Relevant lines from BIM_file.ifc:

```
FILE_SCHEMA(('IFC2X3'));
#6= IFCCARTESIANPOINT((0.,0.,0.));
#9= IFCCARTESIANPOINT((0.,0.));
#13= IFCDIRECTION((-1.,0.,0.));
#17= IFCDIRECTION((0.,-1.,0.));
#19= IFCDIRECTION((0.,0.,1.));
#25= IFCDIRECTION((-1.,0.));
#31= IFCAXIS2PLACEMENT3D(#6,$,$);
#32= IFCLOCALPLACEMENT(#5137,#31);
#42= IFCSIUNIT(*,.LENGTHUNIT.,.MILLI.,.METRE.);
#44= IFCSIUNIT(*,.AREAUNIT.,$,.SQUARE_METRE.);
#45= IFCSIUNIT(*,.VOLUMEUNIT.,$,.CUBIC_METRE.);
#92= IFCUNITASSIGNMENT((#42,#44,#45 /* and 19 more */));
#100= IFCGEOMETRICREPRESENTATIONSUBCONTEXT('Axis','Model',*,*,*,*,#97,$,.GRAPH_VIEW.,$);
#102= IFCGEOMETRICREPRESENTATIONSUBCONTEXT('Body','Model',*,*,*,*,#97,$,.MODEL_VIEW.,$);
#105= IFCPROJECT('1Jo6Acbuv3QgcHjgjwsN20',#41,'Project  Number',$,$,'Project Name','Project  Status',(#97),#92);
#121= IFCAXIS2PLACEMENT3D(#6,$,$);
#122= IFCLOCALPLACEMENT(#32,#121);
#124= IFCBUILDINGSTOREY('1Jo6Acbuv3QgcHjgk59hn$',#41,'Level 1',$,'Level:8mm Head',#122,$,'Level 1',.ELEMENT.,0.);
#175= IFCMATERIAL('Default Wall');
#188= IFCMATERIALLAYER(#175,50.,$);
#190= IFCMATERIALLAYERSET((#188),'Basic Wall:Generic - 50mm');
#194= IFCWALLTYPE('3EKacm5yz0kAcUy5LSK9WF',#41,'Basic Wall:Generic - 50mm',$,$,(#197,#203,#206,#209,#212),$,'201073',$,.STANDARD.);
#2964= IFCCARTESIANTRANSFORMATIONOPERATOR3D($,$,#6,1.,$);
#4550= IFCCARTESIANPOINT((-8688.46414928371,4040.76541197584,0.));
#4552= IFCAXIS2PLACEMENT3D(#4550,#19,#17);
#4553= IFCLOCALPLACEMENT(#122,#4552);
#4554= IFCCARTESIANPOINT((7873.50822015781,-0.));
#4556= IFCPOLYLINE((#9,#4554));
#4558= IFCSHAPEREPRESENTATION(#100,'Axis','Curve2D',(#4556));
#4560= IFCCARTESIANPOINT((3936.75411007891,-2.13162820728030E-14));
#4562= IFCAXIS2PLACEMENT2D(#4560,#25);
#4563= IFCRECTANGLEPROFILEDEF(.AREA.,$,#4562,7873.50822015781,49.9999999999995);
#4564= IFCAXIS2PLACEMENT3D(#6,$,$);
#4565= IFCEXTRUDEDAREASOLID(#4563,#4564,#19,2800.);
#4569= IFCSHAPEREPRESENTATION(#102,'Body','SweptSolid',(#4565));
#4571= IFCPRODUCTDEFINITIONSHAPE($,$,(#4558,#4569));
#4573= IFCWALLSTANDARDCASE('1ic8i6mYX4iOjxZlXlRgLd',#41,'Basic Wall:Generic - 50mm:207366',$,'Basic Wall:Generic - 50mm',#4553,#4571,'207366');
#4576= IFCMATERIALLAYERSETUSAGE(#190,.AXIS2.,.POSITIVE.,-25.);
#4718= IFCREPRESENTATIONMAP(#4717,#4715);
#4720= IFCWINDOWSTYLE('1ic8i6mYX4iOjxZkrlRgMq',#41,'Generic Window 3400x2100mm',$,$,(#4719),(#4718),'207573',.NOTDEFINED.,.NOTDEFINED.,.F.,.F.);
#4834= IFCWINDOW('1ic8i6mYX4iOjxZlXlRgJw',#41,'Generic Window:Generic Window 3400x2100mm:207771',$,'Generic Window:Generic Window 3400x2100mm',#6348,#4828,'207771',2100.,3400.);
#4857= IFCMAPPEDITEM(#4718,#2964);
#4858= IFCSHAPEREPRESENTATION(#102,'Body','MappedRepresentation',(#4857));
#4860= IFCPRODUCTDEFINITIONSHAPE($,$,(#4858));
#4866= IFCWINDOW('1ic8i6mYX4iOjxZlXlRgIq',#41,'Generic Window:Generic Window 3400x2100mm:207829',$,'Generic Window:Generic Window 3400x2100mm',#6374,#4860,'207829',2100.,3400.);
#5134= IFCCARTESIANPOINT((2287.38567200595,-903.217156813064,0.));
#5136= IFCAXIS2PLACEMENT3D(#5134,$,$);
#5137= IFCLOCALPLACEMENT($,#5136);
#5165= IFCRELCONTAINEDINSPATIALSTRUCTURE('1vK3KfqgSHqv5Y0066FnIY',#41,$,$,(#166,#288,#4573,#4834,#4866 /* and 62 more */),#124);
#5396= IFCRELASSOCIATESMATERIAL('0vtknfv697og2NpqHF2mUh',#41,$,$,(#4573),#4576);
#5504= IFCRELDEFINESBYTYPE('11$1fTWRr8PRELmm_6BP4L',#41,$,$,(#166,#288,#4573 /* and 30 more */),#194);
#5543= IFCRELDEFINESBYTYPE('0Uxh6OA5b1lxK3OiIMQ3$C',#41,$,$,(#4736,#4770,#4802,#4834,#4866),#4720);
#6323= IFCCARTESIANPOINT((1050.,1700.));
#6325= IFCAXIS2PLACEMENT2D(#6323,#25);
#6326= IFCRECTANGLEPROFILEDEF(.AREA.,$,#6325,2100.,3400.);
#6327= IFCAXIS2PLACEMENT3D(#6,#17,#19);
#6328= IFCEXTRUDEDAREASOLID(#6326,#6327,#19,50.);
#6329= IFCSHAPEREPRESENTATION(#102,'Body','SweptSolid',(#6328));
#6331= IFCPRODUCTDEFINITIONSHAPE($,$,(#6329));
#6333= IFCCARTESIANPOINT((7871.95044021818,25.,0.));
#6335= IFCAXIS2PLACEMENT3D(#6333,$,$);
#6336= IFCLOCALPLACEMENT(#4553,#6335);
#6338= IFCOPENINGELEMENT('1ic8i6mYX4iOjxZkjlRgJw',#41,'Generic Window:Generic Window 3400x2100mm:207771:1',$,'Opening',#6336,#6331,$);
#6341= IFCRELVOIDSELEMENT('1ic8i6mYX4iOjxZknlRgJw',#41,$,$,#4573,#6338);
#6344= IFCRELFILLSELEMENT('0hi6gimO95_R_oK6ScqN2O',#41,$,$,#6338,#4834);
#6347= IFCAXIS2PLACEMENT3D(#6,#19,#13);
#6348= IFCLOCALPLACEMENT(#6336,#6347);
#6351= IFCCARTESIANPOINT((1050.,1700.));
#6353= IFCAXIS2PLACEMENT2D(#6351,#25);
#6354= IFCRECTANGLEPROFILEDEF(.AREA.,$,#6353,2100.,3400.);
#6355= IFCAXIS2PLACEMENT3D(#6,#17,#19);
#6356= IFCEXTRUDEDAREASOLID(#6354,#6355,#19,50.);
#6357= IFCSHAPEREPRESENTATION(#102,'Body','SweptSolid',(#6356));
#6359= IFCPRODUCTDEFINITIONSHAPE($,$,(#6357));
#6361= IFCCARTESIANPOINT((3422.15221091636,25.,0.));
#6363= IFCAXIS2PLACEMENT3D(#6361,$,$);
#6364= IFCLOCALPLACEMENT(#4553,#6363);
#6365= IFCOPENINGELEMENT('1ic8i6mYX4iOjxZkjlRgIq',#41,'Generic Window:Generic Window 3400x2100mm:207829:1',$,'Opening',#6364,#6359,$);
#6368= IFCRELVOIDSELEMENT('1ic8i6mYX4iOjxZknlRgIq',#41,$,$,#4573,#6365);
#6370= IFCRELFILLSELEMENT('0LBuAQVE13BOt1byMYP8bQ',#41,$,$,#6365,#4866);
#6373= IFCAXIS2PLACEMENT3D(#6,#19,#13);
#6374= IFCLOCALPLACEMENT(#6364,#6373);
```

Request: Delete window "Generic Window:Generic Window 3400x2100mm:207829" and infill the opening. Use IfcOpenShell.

```python
import ifcopenshell
import ifcopenshell.api.feature
import ifcopenshell.api.root
import ifcopenshell.geom
import ifcopenshell.util.shape

model = ifcopenshell.open("BIM_file.ifc")
settings = ifcopenshell.geom.settings()


def volume(element):
    """Net volume in cubic metres, openings subtracted."""
    shape = ifcopenshell.geom.create_shape(settings, element)
    return ifcopenshell.util.shape.get_volume(shape.geometry)


window = model.by_guid("1ic8i6mYX4iOjxZlXlRgIq")
opening = window.FillsVoids[0].RelatingOpeningElement
wall = opening.VoidsElements[0].RelatingBuildingElement
before = volume(wall)

ifcopenshell.api.root.remove_product(model, product=window)
ifcopenshell.api.feature.remove_feature(model, feature=opening)

after = volume(wall)

print(f"wall volume {before:.3f} -> {after:.3f} m3")

model.write("BIM_file_edited.ifc")
```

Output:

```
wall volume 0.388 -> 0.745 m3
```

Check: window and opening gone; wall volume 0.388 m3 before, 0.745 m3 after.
